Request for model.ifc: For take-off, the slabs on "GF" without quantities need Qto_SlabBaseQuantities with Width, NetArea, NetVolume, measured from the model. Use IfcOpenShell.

First a look at what the model holds.

```python
import ifcopenshell
import ifcopenshell.util.element
import ifcopenshell.util.unit

model = ifcopenshell.open("model.ifc")
print(model.schema)
for unit_type in ("LENGTHUNIT", "AREAUNIT", "VOLUMEUNIT"):
    print(unit_type, ifcopenshell.util.unit.calculate_unit_scale(model, unit_type))
storey = next(s for s in model.by_type("IfcBuildingStorey") if s.Name == "GF")
slabs = [e for e in ifcopenshell.util.element.get_decomposition(storey) if e.is_a("IfcSlab")]
for e in sorted(slabs, key=lambda e: e.id()):
    print(e.id(), e.is_a(), e.Name, list(ifcopenshell.util.element.get_psets(e, qtos_only=True)), sep=" | ")
```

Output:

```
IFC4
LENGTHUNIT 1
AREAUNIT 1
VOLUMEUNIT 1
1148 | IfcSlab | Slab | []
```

```python
import ifcopenshell
import ifcopenshell.api.pset
import ifcopenshell.geom
import ifcopenshell.util.element
import ifcopenshell.util.shape
import ifcopenshell.util.unit

model = ifcopenshell.open("model.ifc")
unit_scale = ifcopenshell.util.unit.calculate_unit_scale(model)
area_scale = ifcopenshell.util.unit.calculate_unit_scale(model, "AREAUNIT")
volume_scale = ifcopenshell.util.unit.calculate_unit_scale(model, "VOLUMEUNIT")
settings = ifcopenshell.geom.settings()

storey = next(s for s in model.by_type("IfcBuildingStorey") if s.Name == "GF")
slabs = [e for e in ifcopenshell.util.element.get_decomposition(storey) if e.is_a("IfcSlab")]

for e in sorted(slabs, key=lambda e: e.id()):
    if ifcopenshell.util.element.get_psets(e, qtos_only=True, should_inherit=False):
        continue
    # Geometry comes back in metres, in the element's own axes.
    shape = ifcopenshell.geom.create_shape(settings, e)
    values = {
        "Width": ifcopenshell.util.shape.get_z(shape.geometry) / unit_scale,
        "NetArea": ifcopenshell.util.shape.get_footprint_area(shape.geometry) / area_scale,
        "NetVolume": ifcopenshell.util.shape.get_volume(shape.geometry) / volume_scale,
    }
    qto = ifcopenshell.api.pset.add_qto(model, product=e, name="Qto_SlabBaseQuantities")
    ifcopenshell.api.pset.edit_qto(model, qto=qto, properties=values)
    print(e.id(), {k: round(v, 3) for k, v in values.items()})

model.write("model_rev.ifc")
```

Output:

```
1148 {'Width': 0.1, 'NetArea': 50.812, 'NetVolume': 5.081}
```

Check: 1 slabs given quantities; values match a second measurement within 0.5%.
